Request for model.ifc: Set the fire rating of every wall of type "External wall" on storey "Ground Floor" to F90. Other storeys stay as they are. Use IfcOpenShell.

First a look at what the model holds.

```python
import ifcopenshell
import ifcopenshell.util.element

model = ifcopenshell.open("model.ifc")
print(model.schema)
storey = next(s for s in model.by_type("IfcBuildingStorey") if s.Name == "Ground Floor")
walls = [e for e in ifcopenshell.util.element.get_decomposition(storey) if e.is_a("IfcWall")]
seen = {}
for e in walls:
    element_type = ifcopenshell.util.element.get_type(e)
    key = (element_type.Name if element_type != e and element_type else None, ifcopenshell.util.element.get_pset(e, "Pset_WallCommon", "FireRating"))
    seen[key] = seen.get(key, 0) + 1
for (name, value), count in sorted(seen.items(), key=str):
    print(count, "x", name, "|", value)
```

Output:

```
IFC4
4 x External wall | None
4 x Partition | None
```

```python
import ifcopenshell
import ifcopenshell.api.pset
import ifcopenshell.util.element

model = ifcopenshell.open("model.ifc")

storey = next(s for s in model.by_type("IfcBuildingStorey") if s.Name == "Ground Floor")
walls = [e for e in ifcopenshell.util.element.get_decomposition(storey) if e.is_a("IfcWall")]

count = 0
for e in walls:
    element_type = ifcopenshell.util.element.get_type(e)
    if element_type in (None, e) or element_type.Name != "External wall":
        continue
    # add_pset returns the element's existing set when there is one.
    pset = ifcopenshell.api.pset.add_pset(model, product=e, name="Pset_WallCommon")
    ifcopenshell.api.pset.edit_pset(model, pset=pset, properties={"FireRating": "F90"})
    count += 1

print(count, "walls updated")

model.write("model-out.ifc")
```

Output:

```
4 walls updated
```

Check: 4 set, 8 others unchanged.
